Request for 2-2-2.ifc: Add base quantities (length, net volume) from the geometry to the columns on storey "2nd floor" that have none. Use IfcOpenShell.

First a look at what the model holds.

```python
import ifcopenshell
import ifcopenshell.util.element
import ifcopenshell.util.unit

model = ifcopenshell.open("2-2-2.ifc")
print(model.schema)
for unit_type in ("LENGTHUNIT", "AREAUNIT", "VOLUMEUNIT"):
    print(unit_type, ifcopenshell.util.unit.calculate_unit_scale(model, unit_type))
storey = next(s for s in model.by_type("IfcBuildingStorey") if s.Name == "2nd floor")
columns = [e for e in ifcopenshell.util.element.get_decomposition(storey) if e.is_a("IfcColumn")]
for e in sorted(columns, key=lambda e: e.id()):
    print(e.id(), e.is_a(), e.Name, list(ifcopenshell.util.element.get_psets(e, qtos_only=True)), sep=" | ")
```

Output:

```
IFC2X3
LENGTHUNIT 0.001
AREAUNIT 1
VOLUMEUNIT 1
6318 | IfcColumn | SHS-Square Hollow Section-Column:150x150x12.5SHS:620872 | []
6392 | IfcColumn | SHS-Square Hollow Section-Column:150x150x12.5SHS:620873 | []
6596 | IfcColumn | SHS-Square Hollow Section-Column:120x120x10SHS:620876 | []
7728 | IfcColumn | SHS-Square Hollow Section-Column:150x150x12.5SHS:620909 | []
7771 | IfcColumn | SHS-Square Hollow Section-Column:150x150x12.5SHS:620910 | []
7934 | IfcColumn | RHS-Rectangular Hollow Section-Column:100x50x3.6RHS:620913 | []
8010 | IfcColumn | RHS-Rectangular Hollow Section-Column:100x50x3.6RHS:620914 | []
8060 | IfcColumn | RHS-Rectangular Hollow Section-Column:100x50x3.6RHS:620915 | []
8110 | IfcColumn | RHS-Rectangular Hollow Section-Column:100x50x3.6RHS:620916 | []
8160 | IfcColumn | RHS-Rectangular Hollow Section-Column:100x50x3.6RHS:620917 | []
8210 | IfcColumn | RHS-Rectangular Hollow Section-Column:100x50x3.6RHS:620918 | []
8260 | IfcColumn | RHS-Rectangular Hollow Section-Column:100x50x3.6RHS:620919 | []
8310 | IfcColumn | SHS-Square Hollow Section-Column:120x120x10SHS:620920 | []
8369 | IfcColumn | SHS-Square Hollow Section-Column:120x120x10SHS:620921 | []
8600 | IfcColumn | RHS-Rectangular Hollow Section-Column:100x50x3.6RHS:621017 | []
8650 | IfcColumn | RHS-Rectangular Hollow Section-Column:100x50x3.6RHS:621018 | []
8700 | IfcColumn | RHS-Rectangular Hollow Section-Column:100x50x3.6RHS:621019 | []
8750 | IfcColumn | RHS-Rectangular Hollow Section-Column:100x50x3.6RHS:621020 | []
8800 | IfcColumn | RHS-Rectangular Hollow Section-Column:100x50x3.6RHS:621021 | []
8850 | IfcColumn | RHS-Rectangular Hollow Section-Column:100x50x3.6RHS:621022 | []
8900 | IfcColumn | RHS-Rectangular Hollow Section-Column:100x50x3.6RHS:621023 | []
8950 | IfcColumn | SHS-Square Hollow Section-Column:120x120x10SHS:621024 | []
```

```python
import ifcopenshell
import ifcopenshell.api.pset
import ifcopenshell.geom
import ifcopenshell.util.element
import ifcopenshell.util.shape
import ifcopenshell.util.unit

model = ifcopenshell.open("2-2-2.ifc")
unit_scale = ifcopenshell.util.unit.calculate_unit_scale(model)
volume_scale = ifcopenshell.util.unit.calculate_unit_scale(model, "VOLUMEUNIT")
settings = ifcopenshell.geom.settings()

storey = next(s for s in model.by_type("IfcBuildingStorey") if s.Name == "2nd floor")
columns = [e for e in ifcopenshell.util.element.get_decomposition(storey) if e.is_a("IfcColumn")]

for e in sorted(columns, key=lambda e: e.id()):
    if ifcopenshell.util.element.get_psets(e, qtos_only=True, should_inherit=False):
        continue
    # Geometry comes back in metres, in the element's own axes.
    shape = ifcopenshell.geom.create_shape(settings, e)
    values = {
        "Length": ifcopenshell.util.shape.get_z(shape.geometry) / unit_scale,
        "NetVolume": ifcopenshell.util.shape.get_volume(shape.geometry) / volume_scale,
    }
    qto = ifcopenshell.api.pset.add_qto(model, product=e, name="BaseQuantities")
    ifcopenshell.api.pset.edit_qto(model, qto=qto, properties=values)
    print(e.id(), {k: round(v, 3) for k, v in values.items()})

model.write("2-2-2_edited.ifc")
```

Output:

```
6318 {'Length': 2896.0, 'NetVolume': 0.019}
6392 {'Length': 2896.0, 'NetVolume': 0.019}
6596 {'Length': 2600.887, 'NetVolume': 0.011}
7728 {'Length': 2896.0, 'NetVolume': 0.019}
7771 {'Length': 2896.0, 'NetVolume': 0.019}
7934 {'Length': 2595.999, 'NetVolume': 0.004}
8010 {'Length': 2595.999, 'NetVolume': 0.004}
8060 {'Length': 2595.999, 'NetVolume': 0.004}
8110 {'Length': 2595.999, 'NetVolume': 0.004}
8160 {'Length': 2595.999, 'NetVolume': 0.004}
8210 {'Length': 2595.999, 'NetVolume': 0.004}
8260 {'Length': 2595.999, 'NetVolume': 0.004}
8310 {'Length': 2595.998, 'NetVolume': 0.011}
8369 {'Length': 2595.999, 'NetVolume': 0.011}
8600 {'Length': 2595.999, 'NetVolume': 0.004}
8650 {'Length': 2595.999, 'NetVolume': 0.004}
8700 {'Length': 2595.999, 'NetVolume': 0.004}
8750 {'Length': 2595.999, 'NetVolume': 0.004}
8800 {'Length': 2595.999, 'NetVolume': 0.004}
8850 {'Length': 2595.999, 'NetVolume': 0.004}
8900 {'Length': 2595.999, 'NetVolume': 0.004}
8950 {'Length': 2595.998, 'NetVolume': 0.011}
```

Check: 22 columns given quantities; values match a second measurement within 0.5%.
